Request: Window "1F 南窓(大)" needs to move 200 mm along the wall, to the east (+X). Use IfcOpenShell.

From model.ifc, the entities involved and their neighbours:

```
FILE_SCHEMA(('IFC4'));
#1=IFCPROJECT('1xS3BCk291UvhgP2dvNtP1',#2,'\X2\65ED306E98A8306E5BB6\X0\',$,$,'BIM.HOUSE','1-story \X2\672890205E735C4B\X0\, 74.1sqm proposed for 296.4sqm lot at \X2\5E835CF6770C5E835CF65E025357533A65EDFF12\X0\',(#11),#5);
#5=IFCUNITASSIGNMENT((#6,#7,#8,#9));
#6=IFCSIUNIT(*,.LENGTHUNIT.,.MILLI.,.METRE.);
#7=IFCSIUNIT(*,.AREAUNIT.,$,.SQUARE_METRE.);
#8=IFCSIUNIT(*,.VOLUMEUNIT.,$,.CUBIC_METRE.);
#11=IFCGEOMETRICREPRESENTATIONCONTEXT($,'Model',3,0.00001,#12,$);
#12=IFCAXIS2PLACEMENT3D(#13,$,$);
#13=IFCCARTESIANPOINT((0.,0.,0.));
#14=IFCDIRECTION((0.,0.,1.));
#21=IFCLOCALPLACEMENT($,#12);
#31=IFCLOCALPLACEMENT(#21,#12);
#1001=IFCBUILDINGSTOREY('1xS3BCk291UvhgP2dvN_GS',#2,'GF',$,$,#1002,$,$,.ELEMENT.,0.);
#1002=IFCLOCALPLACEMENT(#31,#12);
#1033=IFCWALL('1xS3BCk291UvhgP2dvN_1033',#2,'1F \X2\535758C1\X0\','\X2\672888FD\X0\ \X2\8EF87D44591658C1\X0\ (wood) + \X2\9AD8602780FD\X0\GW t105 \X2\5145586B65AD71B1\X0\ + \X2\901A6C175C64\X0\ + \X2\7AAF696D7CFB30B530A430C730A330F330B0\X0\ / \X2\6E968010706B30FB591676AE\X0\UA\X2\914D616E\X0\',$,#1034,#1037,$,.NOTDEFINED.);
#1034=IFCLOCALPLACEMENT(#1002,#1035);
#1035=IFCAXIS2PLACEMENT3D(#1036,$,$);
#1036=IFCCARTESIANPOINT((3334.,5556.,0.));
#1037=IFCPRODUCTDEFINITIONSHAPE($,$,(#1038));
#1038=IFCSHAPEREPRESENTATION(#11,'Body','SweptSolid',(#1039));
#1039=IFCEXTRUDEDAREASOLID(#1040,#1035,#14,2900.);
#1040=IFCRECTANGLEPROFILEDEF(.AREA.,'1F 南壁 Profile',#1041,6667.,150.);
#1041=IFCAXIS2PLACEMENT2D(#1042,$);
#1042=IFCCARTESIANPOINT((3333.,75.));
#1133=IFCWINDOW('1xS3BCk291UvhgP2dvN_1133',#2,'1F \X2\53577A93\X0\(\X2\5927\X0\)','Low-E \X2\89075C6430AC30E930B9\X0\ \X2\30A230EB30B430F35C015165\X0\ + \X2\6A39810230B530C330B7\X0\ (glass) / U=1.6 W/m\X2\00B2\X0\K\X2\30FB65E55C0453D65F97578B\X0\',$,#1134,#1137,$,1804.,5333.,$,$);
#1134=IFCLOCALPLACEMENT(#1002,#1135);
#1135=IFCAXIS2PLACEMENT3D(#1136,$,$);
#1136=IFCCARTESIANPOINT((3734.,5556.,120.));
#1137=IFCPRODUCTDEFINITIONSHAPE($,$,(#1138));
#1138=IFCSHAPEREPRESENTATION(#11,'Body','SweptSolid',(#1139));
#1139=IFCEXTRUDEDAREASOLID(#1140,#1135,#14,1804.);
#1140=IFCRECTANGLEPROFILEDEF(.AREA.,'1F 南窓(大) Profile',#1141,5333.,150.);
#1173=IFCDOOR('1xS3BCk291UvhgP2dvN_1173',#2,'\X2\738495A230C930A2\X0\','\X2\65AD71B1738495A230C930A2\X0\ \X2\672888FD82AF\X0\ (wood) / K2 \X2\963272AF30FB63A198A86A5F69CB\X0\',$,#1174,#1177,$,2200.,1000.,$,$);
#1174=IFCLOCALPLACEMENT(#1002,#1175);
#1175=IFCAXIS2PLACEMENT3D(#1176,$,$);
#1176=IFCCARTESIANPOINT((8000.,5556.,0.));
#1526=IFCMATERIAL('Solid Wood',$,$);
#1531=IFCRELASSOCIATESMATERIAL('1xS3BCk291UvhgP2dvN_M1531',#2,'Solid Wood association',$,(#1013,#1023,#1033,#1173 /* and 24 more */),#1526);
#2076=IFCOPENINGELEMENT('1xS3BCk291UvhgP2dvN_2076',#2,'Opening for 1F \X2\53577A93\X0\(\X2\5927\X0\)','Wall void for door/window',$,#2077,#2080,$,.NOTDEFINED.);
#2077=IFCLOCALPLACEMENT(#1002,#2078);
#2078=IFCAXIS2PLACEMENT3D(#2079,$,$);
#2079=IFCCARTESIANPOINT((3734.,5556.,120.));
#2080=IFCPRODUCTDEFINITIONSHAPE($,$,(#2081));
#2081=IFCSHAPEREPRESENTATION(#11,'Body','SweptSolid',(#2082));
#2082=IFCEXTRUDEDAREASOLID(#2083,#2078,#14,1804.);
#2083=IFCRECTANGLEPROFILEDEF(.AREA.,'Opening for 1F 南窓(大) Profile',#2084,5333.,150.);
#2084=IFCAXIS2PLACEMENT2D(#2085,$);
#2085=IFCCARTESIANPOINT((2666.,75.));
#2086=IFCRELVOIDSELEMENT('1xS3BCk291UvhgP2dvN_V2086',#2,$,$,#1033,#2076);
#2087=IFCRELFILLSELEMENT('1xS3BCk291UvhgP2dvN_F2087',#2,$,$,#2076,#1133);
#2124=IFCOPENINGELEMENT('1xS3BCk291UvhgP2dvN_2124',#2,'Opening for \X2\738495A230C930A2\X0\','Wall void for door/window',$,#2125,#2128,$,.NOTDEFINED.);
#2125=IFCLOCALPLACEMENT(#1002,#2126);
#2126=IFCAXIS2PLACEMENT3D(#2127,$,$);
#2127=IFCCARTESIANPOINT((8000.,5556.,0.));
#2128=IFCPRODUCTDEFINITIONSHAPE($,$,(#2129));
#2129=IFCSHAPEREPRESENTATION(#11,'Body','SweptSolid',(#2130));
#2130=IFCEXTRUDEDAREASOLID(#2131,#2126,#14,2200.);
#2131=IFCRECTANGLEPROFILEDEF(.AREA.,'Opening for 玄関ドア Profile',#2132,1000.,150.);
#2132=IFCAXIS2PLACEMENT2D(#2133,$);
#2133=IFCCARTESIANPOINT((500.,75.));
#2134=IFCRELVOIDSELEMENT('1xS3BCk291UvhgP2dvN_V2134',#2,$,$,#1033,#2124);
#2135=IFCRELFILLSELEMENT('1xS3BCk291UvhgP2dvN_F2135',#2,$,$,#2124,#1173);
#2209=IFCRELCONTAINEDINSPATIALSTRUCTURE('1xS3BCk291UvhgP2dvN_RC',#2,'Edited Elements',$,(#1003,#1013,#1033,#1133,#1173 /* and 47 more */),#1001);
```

```python
import ifcopenshell
import ifcopenshell.api.geometry
import ifcopenshell.util.placement
import ifcopenshell.util.unit

model = ifcopenshell.open("model.ifc")
unit_scale = ifcopenshell.util.unit.calculate_unit_scale(model)

window = model.by_guid("1xS3BCk291UvhgP2dvN_1133")
opening = window.FillsVoids[0].RelatingOpeningElement
wall = opening.VoidsElements[0].RelatingBuildingElement

wall_matrix = ifcopenshell.util.placement.get_local_placement(wall.ObjectPlacement)
shift = wall_matrix[:3, 0] * 0.2 / unit_scale
before = ifcopenshell.util.placement.get_local_placement(window.ObjectPlacement)[:3, 3].copy()

# The window is not placed relative to its opening, so move both.
for product in (opening, window):
    matrix = ifcopenshell.util.placement.get_local_placement(product.ObjectPlacement)
    matrix[:3, 3] += shift
    ifcopenshell.api.geometry.edit_object_placement(model, product=product, matrix=matrix, is_si=False)

after = ifcopenshell.util.placement.get_local_placement(window.ObjectPlacement)[:3, 3]
print("window moved by", (after - before).round(3) + 0.0)

model.write("model_rev.ifc")
```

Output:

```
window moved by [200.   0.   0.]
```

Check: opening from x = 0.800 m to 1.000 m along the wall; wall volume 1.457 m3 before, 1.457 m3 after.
